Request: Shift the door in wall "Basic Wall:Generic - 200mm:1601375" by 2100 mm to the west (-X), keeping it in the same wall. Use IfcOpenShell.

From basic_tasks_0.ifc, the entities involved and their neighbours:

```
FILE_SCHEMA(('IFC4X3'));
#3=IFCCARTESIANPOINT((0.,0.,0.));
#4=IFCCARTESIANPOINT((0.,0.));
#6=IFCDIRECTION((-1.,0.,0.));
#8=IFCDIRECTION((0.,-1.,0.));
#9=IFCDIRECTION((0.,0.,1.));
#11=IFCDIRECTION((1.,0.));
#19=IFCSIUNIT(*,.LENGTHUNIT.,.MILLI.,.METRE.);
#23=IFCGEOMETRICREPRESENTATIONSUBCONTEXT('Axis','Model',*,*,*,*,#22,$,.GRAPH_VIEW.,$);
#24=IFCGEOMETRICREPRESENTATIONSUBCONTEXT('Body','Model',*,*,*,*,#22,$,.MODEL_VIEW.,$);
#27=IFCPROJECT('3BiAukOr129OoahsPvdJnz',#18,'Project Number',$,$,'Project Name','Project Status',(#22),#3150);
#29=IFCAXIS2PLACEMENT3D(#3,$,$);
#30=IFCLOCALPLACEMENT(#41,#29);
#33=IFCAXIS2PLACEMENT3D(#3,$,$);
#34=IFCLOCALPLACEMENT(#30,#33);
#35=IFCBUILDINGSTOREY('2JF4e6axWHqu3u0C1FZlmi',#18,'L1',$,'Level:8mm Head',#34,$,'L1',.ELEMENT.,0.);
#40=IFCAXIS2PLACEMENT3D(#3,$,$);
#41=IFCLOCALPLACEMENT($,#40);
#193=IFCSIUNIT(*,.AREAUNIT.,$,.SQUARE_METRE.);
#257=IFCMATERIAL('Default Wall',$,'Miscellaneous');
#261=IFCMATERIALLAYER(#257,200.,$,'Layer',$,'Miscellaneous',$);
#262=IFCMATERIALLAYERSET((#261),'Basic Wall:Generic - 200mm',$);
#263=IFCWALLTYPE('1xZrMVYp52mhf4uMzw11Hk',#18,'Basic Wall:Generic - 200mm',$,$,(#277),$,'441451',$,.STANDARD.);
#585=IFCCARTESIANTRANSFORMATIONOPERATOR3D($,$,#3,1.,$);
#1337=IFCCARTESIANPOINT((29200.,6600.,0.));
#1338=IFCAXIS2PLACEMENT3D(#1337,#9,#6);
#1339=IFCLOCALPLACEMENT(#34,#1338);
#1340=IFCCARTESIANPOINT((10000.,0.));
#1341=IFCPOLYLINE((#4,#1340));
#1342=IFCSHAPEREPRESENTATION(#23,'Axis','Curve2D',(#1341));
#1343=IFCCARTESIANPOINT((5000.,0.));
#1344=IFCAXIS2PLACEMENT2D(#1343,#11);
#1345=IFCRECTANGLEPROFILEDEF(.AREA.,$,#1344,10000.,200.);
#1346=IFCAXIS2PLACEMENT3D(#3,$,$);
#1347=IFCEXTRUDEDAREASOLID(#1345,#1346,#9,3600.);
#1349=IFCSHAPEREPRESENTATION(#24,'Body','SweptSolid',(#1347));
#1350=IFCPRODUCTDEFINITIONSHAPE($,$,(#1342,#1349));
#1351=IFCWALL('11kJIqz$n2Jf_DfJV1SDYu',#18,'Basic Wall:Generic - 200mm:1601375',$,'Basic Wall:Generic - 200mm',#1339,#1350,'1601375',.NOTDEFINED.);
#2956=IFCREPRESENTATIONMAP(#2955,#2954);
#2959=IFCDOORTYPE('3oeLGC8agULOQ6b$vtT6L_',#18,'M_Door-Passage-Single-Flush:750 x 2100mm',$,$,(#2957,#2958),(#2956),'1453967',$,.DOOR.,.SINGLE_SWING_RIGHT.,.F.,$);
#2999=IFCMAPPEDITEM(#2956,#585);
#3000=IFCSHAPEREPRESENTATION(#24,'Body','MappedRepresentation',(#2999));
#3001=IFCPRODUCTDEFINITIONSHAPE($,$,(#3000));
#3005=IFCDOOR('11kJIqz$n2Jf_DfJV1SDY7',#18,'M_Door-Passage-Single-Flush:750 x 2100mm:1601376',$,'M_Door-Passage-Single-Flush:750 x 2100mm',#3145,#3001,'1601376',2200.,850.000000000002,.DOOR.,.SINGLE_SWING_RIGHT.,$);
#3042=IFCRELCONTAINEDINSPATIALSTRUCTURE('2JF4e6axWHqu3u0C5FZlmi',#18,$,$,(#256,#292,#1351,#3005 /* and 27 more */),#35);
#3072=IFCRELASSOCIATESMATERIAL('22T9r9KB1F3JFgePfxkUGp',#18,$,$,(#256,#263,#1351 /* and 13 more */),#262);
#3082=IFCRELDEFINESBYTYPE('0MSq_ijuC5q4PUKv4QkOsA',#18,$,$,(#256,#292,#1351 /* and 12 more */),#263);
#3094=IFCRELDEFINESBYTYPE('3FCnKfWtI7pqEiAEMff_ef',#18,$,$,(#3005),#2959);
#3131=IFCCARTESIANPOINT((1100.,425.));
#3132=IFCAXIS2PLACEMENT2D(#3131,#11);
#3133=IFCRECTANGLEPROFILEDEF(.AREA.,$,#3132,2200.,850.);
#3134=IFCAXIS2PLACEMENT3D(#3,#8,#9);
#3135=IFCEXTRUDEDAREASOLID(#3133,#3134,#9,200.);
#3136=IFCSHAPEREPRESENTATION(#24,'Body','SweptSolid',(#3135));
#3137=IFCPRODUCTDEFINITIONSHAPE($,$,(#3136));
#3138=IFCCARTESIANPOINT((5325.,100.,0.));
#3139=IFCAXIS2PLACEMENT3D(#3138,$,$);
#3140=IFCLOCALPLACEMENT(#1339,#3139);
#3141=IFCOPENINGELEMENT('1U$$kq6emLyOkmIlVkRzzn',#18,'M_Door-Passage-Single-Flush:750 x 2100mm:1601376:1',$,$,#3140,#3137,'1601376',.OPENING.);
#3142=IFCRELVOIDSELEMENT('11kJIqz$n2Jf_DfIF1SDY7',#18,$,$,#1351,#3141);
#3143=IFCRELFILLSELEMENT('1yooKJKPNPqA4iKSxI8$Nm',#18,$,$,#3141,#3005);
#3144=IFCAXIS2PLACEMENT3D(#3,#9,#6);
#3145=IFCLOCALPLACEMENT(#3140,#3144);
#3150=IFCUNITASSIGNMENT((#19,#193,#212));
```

```python
import ifcopenshell
import ifcopenshell.api.geometry
import ifcopenshell.util.placement
import ifcopenshell.util.unit

model = ifcopenshell.open("basic_tasks_0.ifc")
unit_scale = ifcopenshell.util.unit.calculate_unit_scale(model)

door = model.by_guid("11kJIqz$n2Jf_DfJV1SDY7")
opening = door.FillsVoids[0].RelatingOpeningElement
wall = opening.VoidsElements[0].RelatingBuildingElement

wall_matrix = ifcopenshell.util.placement.get_local_placement(wall.ObjectPlacement)
shift = wall_matrix[:3, 0] * 2.1 / unit_scale
before = ifcopenshell.util.placement.get_local_placement(door.ObjectPlacement)[:3, 3].copy()

# The door is placed relative to its opening, so it follows when the opening moves.
matrix = ifcopenshell.util.placement.get_local_placement(opening.ObjectPlacement)
matrix[:3, 3] += shift
ifcopenshell.api.geometry.edit_object_placement(
    model, product=opening, matrix=matrix, is_si=False, should_transform_children=True
)

after = ifcopenshell.util.placement.get_local_placement(door.ObjectPlacement)[:3, 3]
print("door moved by", (after - before).round(3) + 0.0)

model.write("basic_tasks_0_v2.ifc")
```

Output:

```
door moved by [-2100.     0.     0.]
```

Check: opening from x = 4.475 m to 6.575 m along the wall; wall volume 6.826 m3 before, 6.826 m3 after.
